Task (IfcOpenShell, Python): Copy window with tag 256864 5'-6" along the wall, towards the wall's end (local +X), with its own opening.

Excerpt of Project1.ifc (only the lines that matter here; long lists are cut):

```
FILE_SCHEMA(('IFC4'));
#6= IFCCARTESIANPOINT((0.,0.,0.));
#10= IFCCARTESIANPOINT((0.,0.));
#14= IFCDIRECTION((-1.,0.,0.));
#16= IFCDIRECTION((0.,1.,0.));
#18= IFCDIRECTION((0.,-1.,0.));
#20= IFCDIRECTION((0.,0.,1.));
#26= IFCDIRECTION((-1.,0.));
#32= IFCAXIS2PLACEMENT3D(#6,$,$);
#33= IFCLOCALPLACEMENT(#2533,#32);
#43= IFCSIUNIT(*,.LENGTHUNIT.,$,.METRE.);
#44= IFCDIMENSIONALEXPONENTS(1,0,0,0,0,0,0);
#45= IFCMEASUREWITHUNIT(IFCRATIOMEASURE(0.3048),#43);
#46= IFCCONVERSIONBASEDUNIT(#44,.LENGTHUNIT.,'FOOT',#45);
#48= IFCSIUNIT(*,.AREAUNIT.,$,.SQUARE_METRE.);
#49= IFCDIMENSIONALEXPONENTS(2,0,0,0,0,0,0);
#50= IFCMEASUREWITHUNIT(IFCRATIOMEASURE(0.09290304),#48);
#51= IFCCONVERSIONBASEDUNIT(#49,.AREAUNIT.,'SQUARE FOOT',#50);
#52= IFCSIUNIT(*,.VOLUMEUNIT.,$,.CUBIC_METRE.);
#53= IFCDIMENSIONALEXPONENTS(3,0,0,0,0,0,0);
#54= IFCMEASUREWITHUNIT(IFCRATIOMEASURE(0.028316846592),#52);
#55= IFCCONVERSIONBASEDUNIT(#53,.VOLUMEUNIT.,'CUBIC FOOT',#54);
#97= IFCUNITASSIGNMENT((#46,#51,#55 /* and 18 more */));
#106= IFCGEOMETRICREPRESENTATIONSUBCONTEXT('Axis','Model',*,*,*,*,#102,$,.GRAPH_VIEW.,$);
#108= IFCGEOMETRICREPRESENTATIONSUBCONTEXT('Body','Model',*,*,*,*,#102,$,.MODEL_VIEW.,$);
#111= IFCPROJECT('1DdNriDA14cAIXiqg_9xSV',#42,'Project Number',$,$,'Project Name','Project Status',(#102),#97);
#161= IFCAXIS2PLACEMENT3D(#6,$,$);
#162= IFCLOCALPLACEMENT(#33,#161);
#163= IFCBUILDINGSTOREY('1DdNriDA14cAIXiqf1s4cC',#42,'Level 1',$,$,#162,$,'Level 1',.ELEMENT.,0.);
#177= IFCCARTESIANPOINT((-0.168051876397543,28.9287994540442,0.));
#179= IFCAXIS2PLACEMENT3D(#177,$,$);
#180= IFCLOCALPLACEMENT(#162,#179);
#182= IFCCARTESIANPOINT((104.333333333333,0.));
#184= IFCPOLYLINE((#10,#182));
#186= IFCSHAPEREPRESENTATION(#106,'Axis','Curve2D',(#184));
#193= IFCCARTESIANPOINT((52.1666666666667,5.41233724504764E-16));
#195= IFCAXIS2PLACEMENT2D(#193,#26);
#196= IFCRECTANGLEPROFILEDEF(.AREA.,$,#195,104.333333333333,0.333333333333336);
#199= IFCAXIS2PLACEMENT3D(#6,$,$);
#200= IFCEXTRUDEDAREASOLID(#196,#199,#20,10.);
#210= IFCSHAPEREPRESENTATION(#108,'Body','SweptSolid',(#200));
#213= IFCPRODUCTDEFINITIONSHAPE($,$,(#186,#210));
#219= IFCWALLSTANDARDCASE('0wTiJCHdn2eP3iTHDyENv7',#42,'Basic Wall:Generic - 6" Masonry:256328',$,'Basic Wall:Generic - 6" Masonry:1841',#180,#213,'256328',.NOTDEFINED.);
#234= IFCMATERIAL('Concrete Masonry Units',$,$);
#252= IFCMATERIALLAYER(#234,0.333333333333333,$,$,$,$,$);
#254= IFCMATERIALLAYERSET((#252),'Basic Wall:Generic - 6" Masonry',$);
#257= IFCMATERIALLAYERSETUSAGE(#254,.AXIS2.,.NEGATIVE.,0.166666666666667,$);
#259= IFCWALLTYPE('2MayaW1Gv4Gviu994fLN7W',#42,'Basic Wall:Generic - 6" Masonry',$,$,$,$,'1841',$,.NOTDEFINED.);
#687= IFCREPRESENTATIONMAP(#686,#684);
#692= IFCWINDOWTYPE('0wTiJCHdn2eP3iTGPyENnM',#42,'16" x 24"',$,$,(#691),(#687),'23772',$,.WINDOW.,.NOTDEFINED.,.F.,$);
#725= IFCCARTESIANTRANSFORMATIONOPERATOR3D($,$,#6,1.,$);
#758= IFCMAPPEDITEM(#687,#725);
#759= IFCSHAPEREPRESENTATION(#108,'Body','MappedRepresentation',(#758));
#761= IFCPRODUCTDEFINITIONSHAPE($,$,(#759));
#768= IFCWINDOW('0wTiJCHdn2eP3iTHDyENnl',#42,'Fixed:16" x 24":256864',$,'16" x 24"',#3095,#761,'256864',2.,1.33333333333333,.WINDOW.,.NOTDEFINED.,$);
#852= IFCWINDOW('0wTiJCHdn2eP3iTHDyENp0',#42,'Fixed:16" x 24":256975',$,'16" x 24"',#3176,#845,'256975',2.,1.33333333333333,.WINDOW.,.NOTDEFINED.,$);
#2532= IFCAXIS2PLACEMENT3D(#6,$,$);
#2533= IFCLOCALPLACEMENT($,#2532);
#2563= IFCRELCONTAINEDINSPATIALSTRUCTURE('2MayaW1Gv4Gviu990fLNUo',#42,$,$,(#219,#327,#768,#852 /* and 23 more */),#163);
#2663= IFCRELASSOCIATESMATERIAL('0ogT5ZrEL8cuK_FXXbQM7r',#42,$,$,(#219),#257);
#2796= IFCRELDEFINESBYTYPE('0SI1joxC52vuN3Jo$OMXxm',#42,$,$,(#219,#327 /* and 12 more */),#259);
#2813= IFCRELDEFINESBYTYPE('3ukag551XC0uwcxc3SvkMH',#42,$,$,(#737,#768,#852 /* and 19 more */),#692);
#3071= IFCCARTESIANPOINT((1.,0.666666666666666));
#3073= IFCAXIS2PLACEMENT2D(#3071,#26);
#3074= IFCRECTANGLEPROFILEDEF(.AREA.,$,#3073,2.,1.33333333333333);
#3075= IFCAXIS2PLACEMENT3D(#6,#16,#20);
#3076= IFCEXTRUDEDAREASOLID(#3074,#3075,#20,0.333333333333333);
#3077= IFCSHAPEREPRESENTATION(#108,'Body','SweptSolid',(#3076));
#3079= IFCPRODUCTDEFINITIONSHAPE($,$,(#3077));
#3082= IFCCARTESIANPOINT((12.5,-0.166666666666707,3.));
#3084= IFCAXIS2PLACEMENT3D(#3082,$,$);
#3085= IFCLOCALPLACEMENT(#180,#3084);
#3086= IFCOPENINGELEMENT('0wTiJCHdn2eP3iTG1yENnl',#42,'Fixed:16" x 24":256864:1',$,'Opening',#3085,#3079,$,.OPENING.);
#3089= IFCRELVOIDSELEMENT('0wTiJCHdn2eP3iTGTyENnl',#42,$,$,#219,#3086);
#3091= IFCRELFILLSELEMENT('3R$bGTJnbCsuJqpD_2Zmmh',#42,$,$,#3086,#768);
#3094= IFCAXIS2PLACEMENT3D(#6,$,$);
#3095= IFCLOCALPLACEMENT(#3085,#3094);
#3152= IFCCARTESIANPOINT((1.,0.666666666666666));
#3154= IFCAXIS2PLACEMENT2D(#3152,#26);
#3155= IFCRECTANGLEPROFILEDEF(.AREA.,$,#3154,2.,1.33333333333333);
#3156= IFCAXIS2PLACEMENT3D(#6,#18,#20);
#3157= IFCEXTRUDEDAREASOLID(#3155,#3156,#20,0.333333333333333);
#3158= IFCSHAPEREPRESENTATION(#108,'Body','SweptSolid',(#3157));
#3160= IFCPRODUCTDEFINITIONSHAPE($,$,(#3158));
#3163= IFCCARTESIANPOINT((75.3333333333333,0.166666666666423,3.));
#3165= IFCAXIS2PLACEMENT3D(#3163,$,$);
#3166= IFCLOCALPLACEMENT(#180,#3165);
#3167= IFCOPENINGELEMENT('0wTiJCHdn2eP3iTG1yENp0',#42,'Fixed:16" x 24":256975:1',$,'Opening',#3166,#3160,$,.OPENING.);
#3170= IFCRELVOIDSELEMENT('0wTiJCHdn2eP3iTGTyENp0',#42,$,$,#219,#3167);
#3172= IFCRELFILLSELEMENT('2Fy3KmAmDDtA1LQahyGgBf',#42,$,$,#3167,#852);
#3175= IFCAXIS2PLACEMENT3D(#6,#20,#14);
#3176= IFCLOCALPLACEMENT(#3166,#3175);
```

```python
import ifcopenshell
import ifcopenshell.api.feature
import ifcopenshell.api.geometry
import ifcopenshell.api.root
import ifcopenshell.geom
import ifcopenshell.util.element
import ifcopenshell.util.placement
import ifcopenshell.util.shape
import ifcopenshell.util.unit

model = ifcopenshell.open("Project1.ifc")
unit_scale = ifcopenshell.util.unit.calculate_unit_scale(model)
settings = ifcopenshell.geom.settings()


def volume(element):
    """Net volume in cubic metres, openings subtracted."""
    shape = ifcopenshell.geom.create_shape(settings, element)
    return ifcopenshell.util.shape.get_volume(shape.geometry)


def reuse_history(source, copy):
    """copy_class also copies each property set's owner history, people and application; keep the originals."""
    for rel in copy.IsDefinedBy:
        if rel.is_a("IfcRelDefinesByProperties") and (history := rel.RelatingPropertyDefinition.OwnerHistory):
            rel.RelatingPropertyDefinition.OwnerHistory = source.OwnerHistory
            ifcopenshell.util.element.remove_deep2(model, history)


window = model.by_guid("0wTiJCHdn2eP3iTHDyENnl")
opening = window.FillsVoids[0].RelatingOpeningElement
wall = opening.VoidsElements[0].RelatingBuildingElement
before = volume(wall)
shift = ifcopenshell.util.placement.get_local_placement(wall.ObjectPlacement)[:3, 0] * 66 * 0.0254 / unit_scale

# copy_class copies the void relationship, type, container and properties, but no geometry.
new_opening = ifcopenshell.api.root.copy_class(model, product=opening)
new_opening.Representation = ifcopenshell.util.element.copy_deep(
    model, opening.Representation, exclude=["IfcGeometricRepresentationContext", "IfcRepresentationMap"]
)
new_opening.Name = 'Fixed:16" x 24"'
new_window = ifcopenshell.api.root.copy_class(model, product=window)
new_window.Representation = ifcopenshell.util.element.copy_deep(
    model, window.Representation, exclude=["IfcGeometricRepresentationContext", "IfcRepresentationMap"]
)
new_window.Name = 'Fixed:16" x 24"'
new_window.Tag = None
reuse_history(window, new_window)
ifcopenshell.api.feature.add_filling(model, opening=new_opening, element=new_window)

for old, new in ((opening, new_opening), (window, new_window)):
    matrix = ifcopenshell.util.placement.get_local_placement(old.ObjectPlacement)
    matrix[:3, 3] += shift
    ifcopenshell.api.geometry.edit_object_placement(model, product=new, matrix=matrix, is_si=False)

after = volume(wall)

print(f"wall volume {before:.3f} -> {after:.3f} m3")

model.write("Project1_rev.ifc")
```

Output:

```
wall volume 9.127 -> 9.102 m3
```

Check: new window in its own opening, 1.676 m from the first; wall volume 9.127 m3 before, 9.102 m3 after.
